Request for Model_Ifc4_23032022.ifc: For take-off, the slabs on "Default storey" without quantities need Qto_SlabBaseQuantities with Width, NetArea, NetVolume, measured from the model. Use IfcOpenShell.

First a look at what the model holds.

```python
import ifcopenshell
import ifcopenshell.util.element
import ifcopenshell.util.unit

model = ifcopenshell.open("Model_Ifc4_23032022.ifc")
print(model.schema)
for unit_type in ("LENGTHUNIT", "AREAUNIT", "VOLUMEUNIT"):
    print(unit_type, ifcopenshell.util.unit.calculate_unit_scale(model, unit_type))
storey = next(s for s in model.by_type("IfcBuildingStorey") if s.Name == "Default storey")
slabs = [e for e in ifcopenshell.util.element.get_decomposition(storey) if e.is_a("IfcSlab")]
for e in sorted(slabs, key=lambda e: e.id()):
    print(e.id(), e.is_a(), e.Name, list(ifcopenshell.util.element.get_psets(e, qtos_only=True)), sep=" | ")
```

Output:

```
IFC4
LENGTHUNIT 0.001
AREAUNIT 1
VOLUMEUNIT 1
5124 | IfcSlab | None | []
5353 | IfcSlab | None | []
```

```python
import ifcopenshell
import ifcopenshell.api.pset
import ifcopenshell.geom
import ifcopenshell.util.element
import ifcopenshell.util.shape
import ifcopenshell.util.unit

model = ifcopenshell.open("Model_Ifc4_23032022.ifc")
unit_scale = ifcopenshell.util.unit.calculate_unit_scale(model)
area_scale = ifcopenshell.util.unit.calculate_unit_scale(model, "AREAUNIT")
volume_scale = ifcopenshell.util.unit.calculate_unit_scale(model, "VOLUMEUNIT")
settings = ifcopenshell.geom.settings()

storey = next(s for s in model.by_type("IfcBuildingStorey") if s.Name == "Default storey")
slabs = [e for e in ifcopenshell.util.element.get_decomposition(storey) if e.is_a("IfcSlab")]

for e in sorted(slabs, key=lambda e: e.id()):
    if ifcopenshell.util.element.get_psets(e, qtos_only=True, should_inherit=False):
        continue
    # Geometry comes back in metres, in the element's own axes.
    shape = ifcopenshell.geom.create_shape(settings, e)
    values = {
        "Width": ifcopenshell.util.shape.get_z(shape.geometry) / unit_scale,
        "NetArea": ifcopenshell.util.shape.get_footprint_area(shape.geometry) / area_scale,
        "NetVolume": ifcopenshell.util.shape.get_volume(shape.geometry) / volume_scale,
    }
    qto = ifcopenshell.api.pset.add_qto(model, product=e, name="Qto_SlabBaseQuantities")
    ifcopenshell.api.pset.edit_qto(model, qto=qto, properties=values)
    print(e.id(), {k: round(v, 3) for k, v in values.items()})

model.write("Model_Ifc4_23032022_edited.ifc")
```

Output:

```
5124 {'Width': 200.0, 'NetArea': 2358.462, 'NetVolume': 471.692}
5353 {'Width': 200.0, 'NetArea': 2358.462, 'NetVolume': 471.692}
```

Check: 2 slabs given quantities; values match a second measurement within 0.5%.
